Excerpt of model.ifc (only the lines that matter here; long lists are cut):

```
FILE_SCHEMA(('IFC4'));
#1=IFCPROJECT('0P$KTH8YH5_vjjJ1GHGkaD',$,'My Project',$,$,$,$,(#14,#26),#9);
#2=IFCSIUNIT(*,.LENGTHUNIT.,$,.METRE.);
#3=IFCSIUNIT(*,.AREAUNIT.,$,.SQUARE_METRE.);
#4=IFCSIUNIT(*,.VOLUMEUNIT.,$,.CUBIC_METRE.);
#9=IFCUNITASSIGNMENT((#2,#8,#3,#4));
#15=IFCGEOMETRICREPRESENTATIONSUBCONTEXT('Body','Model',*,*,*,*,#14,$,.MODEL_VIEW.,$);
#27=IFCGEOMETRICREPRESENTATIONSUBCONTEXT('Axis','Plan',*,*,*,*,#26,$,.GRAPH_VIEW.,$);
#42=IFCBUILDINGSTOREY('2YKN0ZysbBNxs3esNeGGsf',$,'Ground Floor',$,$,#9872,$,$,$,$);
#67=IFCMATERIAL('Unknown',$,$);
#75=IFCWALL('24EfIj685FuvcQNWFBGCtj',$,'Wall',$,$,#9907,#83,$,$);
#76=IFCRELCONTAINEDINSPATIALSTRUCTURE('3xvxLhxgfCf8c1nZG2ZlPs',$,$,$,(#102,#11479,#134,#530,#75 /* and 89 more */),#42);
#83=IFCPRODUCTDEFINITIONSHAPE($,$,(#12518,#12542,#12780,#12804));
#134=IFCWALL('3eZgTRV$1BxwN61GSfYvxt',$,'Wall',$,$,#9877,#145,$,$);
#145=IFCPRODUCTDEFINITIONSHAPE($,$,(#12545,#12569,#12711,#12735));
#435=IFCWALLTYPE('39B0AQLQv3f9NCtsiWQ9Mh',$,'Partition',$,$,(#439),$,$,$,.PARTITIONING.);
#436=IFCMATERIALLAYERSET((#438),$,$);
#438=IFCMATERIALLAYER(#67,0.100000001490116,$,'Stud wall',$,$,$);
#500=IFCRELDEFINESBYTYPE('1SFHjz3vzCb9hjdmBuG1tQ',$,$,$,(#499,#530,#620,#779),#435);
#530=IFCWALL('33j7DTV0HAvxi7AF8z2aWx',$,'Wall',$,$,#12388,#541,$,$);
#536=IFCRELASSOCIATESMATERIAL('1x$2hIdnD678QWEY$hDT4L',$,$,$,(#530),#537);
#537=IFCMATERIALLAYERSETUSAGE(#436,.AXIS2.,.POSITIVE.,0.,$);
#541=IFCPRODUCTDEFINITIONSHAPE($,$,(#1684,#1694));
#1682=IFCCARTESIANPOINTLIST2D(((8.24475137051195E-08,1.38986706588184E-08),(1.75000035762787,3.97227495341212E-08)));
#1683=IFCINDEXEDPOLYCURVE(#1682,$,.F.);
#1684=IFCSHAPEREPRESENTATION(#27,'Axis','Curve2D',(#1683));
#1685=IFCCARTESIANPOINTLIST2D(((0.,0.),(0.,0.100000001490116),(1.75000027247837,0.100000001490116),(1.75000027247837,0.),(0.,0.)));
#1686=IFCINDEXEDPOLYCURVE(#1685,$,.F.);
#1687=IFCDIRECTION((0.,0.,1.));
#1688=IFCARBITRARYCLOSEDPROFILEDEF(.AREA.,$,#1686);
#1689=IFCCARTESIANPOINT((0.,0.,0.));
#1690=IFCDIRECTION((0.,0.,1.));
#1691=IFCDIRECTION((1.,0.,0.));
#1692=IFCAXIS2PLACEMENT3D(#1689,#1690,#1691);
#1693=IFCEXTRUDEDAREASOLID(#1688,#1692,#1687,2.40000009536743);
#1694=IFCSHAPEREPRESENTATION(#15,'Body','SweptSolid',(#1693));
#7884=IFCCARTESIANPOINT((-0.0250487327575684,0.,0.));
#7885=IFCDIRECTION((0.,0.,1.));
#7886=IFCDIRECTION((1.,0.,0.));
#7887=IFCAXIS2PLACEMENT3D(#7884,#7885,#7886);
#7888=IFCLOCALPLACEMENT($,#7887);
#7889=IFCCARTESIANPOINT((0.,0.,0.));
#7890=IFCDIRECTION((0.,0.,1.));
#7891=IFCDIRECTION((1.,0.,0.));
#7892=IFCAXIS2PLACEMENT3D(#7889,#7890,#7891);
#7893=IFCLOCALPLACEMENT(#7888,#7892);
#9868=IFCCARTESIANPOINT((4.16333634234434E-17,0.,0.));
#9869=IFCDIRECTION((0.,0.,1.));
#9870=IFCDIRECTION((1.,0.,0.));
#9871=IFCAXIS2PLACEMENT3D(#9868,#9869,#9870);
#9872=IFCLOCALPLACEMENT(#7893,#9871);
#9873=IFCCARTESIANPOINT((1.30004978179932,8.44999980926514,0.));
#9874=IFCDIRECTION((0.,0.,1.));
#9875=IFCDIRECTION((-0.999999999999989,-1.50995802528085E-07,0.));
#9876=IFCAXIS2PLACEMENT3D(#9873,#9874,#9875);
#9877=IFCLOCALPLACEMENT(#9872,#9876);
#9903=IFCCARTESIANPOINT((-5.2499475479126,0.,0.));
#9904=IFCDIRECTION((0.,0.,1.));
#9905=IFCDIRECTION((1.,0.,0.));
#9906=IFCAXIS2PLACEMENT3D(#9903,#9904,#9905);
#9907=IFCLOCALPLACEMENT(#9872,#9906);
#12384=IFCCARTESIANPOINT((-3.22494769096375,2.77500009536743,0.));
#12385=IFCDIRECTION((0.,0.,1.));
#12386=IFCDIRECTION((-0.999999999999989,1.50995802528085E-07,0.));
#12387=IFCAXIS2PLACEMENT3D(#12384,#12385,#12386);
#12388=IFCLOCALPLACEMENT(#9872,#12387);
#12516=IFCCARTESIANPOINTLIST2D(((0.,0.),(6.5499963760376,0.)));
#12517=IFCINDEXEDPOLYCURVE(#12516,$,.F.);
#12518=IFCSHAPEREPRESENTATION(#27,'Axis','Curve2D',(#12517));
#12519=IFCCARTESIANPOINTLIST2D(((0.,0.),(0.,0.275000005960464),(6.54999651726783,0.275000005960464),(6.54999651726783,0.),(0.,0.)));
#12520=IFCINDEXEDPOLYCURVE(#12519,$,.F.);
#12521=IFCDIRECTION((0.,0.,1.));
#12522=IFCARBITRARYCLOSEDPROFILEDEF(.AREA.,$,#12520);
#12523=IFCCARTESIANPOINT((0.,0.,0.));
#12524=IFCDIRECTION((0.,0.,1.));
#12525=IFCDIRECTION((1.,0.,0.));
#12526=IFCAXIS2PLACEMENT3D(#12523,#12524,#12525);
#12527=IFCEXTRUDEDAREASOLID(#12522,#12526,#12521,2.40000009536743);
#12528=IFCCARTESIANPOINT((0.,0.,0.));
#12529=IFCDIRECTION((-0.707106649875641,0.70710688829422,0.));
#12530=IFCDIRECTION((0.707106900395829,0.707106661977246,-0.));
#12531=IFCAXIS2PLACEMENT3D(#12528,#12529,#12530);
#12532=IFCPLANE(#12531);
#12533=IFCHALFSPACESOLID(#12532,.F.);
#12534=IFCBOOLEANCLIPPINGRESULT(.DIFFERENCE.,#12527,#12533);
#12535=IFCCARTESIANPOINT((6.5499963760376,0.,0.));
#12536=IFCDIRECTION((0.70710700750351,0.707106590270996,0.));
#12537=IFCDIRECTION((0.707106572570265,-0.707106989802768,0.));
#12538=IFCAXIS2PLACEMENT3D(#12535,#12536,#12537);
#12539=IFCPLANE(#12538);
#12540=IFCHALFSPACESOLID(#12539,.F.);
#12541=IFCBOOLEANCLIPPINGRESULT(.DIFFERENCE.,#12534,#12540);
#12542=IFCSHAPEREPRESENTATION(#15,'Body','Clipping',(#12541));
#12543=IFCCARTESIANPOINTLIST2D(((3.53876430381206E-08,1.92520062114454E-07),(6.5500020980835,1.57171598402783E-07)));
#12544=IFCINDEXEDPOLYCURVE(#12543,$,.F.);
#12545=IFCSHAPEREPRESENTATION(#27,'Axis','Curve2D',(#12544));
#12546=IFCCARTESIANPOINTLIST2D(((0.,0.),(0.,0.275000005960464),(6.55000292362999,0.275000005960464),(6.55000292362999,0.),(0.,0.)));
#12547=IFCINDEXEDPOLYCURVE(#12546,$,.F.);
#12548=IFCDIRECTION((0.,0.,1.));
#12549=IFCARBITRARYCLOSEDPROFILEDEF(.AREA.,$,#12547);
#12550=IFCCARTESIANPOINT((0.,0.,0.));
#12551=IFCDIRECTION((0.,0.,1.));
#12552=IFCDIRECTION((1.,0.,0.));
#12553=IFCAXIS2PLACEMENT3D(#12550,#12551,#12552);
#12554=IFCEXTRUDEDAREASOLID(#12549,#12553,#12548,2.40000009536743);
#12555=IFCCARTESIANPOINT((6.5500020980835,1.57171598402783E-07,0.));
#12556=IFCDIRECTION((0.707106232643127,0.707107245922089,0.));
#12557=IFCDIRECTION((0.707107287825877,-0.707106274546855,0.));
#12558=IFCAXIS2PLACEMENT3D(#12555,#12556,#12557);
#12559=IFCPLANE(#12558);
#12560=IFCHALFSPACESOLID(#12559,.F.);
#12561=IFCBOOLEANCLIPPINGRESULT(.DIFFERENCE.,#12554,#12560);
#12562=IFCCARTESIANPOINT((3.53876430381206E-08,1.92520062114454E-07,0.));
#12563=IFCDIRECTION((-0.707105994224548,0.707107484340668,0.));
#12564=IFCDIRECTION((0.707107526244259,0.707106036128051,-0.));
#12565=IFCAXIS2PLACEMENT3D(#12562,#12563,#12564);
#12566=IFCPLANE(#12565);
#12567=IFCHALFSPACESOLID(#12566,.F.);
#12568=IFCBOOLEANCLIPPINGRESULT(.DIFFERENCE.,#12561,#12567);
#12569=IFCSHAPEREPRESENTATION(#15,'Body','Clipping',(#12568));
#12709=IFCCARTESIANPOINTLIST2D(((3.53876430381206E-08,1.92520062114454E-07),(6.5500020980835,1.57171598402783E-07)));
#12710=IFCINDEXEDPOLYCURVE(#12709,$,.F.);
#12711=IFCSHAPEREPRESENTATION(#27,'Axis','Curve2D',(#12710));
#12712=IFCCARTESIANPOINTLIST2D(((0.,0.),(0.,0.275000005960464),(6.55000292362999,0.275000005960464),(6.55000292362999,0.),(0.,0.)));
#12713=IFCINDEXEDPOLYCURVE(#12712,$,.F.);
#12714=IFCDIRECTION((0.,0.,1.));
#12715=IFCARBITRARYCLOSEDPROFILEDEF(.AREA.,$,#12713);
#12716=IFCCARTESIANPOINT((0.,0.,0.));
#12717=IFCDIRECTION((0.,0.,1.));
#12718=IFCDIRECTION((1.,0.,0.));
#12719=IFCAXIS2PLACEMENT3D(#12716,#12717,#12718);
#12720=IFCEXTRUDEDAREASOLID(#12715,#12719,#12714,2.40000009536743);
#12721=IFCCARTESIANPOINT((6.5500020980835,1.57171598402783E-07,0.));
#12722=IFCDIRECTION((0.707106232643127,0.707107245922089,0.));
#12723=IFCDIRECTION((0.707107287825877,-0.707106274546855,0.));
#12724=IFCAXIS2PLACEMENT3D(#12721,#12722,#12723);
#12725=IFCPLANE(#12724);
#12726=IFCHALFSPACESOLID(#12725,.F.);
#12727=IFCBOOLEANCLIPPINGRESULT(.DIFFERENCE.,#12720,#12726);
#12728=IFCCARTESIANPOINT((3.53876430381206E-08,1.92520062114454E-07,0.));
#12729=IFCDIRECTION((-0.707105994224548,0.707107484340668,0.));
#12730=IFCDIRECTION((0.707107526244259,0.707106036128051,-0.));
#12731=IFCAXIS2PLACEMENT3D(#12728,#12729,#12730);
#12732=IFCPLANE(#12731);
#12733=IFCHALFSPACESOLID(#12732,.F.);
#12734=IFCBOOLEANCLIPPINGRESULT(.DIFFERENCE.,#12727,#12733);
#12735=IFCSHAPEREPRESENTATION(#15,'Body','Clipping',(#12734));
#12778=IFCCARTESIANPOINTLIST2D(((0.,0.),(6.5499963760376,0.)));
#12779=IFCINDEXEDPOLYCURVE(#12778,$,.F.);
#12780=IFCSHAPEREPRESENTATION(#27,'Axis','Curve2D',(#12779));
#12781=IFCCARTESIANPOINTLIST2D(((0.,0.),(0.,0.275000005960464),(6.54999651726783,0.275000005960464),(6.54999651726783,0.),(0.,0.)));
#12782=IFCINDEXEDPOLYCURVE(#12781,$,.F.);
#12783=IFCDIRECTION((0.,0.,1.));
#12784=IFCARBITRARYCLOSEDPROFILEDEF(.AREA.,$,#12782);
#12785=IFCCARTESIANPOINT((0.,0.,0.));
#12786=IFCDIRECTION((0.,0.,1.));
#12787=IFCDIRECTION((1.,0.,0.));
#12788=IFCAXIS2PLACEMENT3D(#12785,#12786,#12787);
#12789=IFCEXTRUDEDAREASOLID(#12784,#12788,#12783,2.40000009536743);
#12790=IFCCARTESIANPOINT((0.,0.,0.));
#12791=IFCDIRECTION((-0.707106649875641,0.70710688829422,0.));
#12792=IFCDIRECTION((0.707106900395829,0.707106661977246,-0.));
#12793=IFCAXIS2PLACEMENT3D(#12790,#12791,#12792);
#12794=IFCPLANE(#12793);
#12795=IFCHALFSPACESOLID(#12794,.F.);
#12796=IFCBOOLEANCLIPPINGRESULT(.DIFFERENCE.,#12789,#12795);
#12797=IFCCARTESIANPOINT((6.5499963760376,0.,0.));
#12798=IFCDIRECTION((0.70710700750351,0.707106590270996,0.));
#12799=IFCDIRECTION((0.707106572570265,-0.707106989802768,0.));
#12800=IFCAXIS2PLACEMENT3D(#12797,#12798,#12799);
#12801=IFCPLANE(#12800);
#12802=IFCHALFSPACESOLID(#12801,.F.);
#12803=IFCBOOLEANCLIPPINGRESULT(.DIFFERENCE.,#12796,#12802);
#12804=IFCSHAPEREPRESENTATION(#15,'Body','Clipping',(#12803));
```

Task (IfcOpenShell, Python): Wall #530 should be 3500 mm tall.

```python
import ifcopenshell
import ifcopenshell.geom
import ifcopenshell.util.representation
import ifcopenshell.util.shape
import ifcopenshell.util.unit

model = ifcopenshell.open("model.ifc")
unit_scale = ifcopenshell.util.unit.calculate_unit_scale(model)
settings = ifcopenshell.geom.settings()


def volume(element):
    """Net volume in cubic metres, openings subtracted."""
    shape = ifcopenshell.geom.create_shape(settings, element)
    return ifcopenshell.util.shape.get_volume(shape.geometry)


wall = model.by_id(530)
before = volume(wall)

body = ifcopenshell.util.representation.get_representation(wall, "Model", "Body")
solid = body.Items[0]
old_height = solid.Depth
solid.Depth = 3.5 / unit_scale
after = volume(wall)

print(f"height {old_height:g} -> {solid.Depth:g}, volume {before:.3f} -> {after:.3f} m3")

model.write("model_v2.ifc")
```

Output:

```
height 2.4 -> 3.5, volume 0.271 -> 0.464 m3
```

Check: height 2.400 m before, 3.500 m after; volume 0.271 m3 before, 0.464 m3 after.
